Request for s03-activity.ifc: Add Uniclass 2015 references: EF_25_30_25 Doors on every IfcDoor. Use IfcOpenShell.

First a look at what the model holds.

```python
import ifcopenshell

model = ifcopenshell.open("s03-activity.ifc")
print(model.schema)
print("classifications:", [c.Name for c in model.by_type("IfcClassification")])
for ifc_class in ("IfcDoor", "IfcRoof", "IfcStair", "IfcWall", "IfcWindow"):
    print(ifc_class, len(model.by_type(ifc_class)))
```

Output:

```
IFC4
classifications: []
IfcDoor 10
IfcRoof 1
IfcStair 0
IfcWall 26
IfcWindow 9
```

```python
import ifcopenshell
import ifcopenshell.api.classification

model = ifcopenshell.open("s03-activity.ifc")

system = ifcopenshell.api.classification.add_classification(model, classification="Uniclass 2015")

codes = {
    "IfcDoor": ("EF_25_30_25", "Doors"),
}
for ifc_class, (code, name) in codes.items():
    products = model.by_type(ifc_class)
    ifcopenshell.api.classification.add_reference(
        model, products=products, classification=system, identification=code, name=name
    )
    print(code, len(products))

model.write("s03-activity-out.ifc")
```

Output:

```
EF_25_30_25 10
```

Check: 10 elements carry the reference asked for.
